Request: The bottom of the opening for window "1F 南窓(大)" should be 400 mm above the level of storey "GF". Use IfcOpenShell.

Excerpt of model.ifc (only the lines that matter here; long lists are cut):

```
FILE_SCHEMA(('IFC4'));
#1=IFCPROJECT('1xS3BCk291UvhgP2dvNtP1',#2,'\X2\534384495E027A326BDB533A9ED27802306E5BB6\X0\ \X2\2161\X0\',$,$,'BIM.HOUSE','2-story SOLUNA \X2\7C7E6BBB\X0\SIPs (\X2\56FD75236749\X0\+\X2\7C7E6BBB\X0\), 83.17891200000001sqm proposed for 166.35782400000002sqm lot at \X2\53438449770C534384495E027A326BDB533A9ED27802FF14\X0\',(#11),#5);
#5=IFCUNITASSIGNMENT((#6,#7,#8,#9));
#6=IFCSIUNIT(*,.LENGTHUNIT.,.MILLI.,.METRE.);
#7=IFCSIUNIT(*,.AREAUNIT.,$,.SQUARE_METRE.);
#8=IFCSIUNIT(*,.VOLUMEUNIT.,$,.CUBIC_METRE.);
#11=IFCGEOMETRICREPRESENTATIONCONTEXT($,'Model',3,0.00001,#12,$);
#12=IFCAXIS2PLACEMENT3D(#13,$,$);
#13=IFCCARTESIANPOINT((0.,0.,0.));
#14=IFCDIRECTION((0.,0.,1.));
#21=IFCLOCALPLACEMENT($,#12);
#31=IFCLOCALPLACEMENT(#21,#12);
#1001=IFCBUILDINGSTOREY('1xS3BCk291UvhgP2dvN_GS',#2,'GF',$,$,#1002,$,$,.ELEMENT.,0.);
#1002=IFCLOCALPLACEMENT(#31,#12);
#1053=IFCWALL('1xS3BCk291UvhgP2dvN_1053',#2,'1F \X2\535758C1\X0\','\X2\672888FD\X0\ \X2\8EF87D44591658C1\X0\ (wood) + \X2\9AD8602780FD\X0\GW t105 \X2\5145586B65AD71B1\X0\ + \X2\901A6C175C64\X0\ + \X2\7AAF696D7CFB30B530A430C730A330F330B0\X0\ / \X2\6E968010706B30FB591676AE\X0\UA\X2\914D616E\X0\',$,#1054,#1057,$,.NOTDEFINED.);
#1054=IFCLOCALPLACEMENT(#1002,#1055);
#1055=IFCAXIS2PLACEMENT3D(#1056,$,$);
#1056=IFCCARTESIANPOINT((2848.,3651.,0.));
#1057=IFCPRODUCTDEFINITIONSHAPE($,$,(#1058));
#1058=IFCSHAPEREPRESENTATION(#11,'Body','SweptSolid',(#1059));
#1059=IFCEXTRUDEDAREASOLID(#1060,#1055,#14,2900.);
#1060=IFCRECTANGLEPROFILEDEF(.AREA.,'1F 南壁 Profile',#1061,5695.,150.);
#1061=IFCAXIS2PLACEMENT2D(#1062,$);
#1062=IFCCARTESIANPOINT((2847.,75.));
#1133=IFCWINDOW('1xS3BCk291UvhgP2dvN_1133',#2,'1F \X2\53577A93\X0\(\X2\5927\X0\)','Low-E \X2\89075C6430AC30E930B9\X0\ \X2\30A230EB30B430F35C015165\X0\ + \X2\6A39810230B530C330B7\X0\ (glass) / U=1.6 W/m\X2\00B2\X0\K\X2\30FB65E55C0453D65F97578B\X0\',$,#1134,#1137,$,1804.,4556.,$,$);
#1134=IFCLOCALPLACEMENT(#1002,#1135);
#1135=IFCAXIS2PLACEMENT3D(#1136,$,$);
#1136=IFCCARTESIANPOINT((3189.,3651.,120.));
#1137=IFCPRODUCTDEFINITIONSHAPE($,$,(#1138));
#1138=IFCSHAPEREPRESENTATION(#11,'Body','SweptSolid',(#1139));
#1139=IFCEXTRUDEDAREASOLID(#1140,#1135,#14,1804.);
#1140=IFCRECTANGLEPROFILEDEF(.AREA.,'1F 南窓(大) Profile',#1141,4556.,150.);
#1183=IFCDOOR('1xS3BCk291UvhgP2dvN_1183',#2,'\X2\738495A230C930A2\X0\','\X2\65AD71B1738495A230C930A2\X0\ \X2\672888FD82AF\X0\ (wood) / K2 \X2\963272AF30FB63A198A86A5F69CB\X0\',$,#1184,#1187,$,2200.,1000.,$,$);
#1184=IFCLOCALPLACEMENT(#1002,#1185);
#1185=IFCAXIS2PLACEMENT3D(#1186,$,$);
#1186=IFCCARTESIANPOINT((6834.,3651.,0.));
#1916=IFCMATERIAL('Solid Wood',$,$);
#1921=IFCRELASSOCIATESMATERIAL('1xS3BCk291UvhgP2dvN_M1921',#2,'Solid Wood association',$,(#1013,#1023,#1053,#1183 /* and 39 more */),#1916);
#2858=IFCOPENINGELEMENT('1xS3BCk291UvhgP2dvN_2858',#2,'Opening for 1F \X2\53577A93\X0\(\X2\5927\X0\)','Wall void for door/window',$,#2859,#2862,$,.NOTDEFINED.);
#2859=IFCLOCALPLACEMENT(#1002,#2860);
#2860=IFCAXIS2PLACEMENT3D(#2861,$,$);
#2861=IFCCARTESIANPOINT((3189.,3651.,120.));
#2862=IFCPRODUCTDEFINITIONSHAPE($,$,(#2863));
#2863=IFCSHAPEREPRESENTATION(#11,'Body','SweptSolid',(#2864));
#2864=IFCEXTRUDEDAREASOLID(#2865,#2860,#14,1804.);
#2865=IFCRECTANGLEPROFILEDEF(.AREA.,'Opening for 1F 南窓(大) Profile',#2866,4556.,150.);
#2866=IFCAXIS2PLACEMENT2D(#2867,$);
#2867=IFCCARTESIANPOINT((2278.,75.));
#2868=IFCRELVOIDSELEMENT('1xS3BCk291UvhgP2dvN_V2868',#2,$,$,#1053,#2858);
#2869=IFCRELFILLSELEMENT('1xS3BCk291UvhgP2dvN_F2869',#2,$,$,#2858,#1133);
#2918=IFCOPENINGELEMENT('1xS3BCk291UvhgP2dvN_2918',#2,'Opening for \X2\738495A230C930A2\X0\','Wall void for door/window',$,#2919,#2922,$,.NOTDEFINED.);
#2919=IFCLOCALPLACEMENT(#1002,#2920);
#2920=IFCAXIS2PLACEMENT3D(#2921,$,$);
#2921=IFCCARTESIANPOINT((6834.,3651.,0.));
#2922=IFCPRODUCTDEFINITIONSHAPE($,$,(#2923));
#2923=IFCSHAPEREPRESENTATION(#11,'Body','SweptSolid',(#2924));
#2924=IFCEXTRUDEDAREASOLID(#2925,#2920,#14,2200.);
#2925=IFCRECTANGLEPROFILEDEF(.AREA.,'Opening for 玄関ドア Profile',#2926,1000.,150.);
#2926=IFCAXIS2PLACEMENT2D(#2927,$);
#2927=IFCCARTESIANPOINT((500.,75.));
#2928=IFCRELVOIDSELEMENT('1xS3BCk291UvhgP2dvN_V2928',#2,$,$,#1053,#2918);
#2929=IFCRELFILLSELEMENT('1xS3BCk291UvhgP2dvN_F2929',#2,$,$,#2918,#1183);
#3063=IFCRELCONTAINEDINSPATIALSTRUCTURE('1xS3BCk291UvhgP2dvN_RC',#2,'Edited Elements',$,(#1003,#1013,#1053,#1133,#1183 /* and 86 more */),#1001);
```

```python
import numpy as np
import ifcopenshell
import ifcopenshell.api.geometry
import ifcopenshell.geom
import ifcopenshell.util.element
import ifcopenshell.util.placement
import ifcopenshell.util.shape
import ifcopenshell.util.unit

model = ifcopenshell.open("model.ifc")
unit_scale = ifcopenshell.util.unit.calculate_unit_scale(model)

window = model.by_guid("1xS3BCk291UvhgP2dvN_1133")
opening = window.FillsVoids[0].RelatingOpeningElement
storey = ifcopenshell.util.element.get_container(window, ifc_class="IfcBuildingStorey")
level = ifcopenshell.util.placement.get_local_placement(storey.ObjectPlacement)[2, 3]

# The opening's origin need not be at the sill, so measure its lowest point.
shape = ifcopenshell.geom.create_shape(ifcopenshell.geom.settings(), opening)
bottom = ifcopenshell.util.shape.get_shape_bottom_elevation(shape, shape.geometry) / unit_scale
dz = level + 0.4 / unit_scale - bottom

shift = np.array([0.0, 0.0, dz])
# The window is not placed relative to its opening, so move both.
for product in (opening, window):
    matrix = ifcopenshell.util.placement.get_local_placement(product.ObjectPlacement)
    matrix[:3, 3] += shift
    ifcopenshell.api.geometry.edit_object_placement(model, product=product, matrix=matrix, is_si=False)

print(f"moved by {dz * unit_scale:+.3f} m")

model.write("model_edited.ifc")
```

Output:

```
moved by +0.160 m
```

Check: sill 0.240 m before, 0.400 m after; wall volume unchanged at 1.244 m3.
